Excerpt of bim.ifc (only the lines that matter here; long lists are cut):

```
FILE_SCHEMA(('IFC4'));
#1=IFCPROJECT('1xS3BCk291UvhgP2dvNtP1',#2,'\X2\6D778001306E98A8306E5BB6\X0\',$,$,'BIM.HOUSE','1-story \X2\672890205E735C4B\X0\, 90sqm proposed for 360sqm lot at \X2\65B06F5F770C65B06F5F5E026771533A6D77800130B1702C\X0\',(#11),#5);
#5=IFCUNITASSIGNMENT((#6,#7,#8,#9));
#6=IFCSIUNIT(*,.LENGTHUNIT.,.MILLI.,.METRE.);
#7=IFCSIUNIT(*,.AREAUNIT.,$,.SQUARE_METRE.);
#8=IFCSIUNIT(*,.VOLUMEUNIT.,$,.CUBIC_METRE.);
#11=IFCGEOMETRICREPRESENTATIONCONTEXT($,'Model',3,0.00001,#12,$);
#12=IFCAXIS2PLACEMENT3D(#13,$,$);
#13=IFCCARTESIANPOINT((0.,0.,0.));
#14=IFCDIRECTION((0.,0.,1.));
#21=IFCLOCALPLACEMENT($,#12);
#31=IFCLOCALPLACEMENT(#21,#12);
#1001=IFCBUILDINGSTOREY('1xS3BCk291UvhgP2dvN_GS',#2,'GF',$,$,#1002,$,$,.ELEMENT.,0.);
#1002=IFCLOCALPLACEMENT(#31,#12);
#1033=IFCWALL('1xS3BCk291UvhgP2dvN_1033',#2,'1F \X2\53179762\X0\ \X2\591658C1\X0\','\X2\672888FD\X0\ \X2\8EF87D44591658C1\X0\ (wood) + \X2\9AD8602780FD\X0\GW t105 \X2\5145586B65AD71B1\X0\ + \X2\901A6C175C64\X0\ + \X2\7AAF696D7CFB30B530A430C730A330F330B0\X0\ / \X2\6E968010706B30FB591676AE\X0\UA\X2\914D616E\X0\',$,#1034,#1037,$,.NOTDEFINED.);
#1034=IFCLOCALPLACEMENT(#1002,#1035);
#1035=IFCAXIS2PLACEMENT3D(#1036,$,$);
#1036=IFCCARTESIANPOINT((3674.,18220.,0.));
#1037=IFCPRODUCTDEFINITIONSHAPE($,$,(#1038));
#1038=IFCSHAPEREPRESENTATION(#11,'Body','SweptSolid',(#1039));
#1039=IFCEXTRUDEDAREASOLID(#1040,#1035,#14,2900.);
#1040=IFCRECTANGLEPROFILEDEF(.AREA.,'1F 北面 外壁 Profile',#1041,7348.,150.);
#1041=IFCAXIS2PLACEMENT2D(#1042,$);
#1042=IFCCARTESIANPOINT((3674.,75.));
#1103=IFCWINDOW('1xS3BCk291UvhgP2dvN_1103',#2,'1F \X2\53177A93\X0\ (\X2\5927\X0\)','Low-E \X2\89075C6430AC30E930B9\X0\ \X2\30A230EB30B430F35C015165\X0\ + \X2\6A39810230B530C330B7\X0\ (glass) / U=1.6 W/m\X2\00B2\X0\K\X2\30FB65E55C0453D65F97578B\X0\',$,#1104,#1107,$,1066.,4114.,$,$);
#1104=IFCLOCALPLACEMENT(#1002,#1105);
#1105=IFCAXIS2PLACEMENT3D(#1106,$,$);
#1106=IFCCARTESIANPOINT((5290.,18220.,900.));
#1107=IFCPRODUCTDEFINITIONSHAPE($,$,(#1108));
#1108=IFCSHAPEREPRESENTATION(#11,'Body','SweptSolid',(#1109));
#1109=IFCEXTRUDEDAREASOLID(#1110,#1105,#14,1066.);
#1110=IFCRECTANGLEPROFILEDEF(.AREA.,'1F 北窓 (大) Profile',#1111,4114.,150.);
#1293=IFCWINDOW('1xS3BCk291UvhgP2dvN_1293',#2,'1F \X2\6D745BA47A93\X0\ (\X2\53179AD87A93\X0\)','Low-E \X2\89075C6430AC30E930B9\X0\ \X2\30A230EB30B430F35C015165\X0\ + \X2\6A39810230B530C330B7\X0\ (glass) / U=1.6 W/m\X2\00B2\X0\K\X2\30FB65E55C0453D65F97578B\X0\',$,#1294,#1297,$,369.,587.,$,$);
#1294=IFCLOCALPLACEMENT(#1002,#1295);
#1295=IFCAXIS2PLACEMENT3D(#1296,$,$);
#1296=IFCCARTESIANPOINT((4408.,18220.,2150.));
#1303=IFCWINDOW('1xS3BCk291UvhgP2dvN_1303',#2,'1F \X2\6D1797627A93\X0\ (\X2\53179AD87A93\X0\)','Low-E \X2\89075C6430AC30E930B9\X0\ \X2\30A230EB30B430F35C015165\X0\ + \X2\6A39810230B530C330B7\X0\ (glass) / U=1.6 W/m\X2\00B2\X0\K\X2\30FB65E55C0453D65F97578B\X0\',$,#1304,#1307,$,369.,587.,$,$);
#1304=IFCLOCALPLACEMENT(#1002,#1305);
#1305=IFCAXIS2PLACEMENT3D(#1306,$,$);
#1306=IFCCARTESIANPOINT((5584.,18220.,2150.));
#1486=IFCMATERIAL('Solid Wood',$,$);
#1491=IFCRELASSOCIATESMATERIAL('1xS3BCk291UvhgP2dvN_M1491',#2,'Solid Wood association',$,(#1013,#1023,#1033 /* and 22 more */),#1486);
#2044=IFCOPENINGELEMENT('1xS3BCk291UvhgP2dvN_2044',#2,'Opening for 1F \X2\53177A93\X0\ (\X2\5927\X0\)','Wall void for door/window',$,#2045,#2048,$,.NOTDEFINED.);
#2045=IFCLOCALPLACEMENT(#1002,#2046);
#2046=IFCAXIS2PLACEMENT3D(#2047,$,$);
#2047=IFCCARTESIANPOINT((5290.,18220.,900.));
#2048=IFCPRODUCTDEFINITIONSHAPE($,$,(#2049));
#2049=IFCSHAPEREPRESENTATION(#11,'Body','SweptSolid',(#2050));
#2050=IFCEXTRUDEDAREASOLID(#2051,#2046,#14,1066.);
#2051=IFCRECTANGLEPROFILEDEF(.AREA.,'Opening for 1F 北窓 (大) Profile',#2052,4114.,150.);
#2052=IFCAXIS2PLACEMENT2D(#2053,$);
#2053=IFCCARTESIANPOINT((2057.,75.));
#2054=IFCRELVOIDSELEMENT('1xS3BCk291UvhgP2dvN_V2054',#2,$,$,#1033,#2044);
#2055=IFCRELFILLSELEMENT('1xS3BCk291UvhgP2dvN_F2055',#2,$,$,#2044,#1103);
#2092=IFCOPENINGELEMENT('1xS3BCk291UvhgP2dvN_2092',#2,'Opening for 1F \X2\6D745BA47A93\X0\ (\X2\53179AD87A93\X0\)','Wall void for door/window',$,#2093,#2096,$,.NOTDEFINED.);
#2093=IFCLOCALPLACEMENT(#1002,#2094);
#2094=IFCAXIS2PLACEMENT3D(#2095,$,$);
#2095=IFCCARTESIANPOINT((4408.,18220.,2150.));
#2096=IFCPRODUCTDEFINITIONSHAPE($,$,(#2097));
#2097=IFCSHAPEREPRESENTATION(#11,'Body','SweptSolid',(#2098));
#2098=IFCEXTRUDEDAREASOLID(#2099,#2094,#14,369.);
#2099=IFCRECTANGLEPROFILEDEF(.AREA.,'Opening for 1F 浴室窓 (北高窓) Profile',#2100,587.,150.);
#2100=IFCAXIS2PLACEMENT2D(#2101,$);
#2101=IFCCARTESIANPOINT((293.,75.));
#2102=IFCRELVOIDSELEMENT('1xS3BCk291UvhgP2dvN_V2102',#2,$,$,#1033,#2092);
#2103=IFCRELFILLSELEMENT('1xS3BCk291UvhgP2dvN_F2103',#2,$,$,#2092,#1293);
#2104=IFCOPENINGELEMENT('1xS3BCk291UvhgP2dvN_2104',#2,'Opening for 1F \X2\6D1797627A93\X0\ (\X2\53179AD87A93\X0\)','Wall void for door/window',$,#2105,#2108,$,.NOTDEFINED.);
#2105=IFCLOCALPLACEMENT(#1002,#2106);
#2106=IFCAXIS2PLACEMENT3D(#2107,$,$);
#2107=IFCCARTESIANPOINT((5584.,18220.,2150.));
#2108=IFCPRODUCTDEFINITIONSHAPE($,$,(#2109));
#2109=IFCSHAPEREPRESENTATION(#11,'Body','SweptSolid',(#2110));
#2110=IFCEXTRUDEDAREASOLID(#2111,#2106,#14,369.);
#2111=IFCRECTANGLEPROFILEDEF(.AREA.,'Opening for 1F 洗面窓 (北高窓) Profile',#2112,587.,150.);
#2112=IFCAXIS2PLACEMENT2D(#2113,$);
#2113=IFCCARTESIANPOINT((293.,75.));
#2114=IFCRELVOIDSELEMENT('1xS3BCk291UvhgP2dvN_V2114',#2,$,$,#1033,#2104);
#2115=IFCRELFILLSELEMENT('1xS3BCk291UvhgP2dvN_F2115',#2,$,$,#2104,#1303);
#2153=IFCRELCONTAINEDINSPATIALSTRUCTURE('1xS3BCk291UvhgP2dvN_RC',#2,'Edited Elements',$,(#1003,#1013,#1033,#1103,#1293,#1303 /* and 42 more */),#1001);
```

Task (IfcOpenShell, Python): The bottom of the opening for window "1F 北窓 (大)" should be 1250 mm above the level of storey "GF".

```python
import numpy as np
import ifcopenshell
import ifcopenshell.api.geometry
import ifcopenshell.geom
import ifcopenshell.util.element
import ifcopenshell.util.placement
import ifcopenshell.util.shape
import ifcopenshell.util.unit

model = ifcopenshell.open("bim.ifc")
unit_scale = ifcopenshell.util.unit.calculate_unit_scale(model)

window = model.by_guid("1xS3BCk291UvhgP2dvN_1103")
opening = window.FillsVoids[0].RelatingOpeningElement
storey = ifcopenshell.util.element.get_container(window, ifc_class="IfcBuildingStorey")
level = ifcopenshell.util.placement.get_local_placement(storey.ObjectPlacement)[2, 3]

# The opening's origin need not be at the sill, so measure its lowest point.
shape = ifcopenshell.geom.create_shape(ifcopenshell.geom.settings(), opening)
bottom = ifcopenshell.util.shape.get_shape_bottom_elevation(shape, shape.geometry) / unit_scale
dz = level + 1.25 / unit_scale - bottom

shift = np.array([0.0, 0.0, dz])
# The window is not placed relative to its opening, so move both.
for product in (opening, window):
    matrix = ifcopenshell.util.placement.get_local_placement(product.ObjectPlacement)
    matrix[:3, 3] += shift
    ifcopenshell.api.geometry.edit_object_placement(model, product=product, matrix=matrix, is_si=False)

print(f"moved by {dz * unit_scale:+.3f} m")

model.write("bim-out.ifc")
```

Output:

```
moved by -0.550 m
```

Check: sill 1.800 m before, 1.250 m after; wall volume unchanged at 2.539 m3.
